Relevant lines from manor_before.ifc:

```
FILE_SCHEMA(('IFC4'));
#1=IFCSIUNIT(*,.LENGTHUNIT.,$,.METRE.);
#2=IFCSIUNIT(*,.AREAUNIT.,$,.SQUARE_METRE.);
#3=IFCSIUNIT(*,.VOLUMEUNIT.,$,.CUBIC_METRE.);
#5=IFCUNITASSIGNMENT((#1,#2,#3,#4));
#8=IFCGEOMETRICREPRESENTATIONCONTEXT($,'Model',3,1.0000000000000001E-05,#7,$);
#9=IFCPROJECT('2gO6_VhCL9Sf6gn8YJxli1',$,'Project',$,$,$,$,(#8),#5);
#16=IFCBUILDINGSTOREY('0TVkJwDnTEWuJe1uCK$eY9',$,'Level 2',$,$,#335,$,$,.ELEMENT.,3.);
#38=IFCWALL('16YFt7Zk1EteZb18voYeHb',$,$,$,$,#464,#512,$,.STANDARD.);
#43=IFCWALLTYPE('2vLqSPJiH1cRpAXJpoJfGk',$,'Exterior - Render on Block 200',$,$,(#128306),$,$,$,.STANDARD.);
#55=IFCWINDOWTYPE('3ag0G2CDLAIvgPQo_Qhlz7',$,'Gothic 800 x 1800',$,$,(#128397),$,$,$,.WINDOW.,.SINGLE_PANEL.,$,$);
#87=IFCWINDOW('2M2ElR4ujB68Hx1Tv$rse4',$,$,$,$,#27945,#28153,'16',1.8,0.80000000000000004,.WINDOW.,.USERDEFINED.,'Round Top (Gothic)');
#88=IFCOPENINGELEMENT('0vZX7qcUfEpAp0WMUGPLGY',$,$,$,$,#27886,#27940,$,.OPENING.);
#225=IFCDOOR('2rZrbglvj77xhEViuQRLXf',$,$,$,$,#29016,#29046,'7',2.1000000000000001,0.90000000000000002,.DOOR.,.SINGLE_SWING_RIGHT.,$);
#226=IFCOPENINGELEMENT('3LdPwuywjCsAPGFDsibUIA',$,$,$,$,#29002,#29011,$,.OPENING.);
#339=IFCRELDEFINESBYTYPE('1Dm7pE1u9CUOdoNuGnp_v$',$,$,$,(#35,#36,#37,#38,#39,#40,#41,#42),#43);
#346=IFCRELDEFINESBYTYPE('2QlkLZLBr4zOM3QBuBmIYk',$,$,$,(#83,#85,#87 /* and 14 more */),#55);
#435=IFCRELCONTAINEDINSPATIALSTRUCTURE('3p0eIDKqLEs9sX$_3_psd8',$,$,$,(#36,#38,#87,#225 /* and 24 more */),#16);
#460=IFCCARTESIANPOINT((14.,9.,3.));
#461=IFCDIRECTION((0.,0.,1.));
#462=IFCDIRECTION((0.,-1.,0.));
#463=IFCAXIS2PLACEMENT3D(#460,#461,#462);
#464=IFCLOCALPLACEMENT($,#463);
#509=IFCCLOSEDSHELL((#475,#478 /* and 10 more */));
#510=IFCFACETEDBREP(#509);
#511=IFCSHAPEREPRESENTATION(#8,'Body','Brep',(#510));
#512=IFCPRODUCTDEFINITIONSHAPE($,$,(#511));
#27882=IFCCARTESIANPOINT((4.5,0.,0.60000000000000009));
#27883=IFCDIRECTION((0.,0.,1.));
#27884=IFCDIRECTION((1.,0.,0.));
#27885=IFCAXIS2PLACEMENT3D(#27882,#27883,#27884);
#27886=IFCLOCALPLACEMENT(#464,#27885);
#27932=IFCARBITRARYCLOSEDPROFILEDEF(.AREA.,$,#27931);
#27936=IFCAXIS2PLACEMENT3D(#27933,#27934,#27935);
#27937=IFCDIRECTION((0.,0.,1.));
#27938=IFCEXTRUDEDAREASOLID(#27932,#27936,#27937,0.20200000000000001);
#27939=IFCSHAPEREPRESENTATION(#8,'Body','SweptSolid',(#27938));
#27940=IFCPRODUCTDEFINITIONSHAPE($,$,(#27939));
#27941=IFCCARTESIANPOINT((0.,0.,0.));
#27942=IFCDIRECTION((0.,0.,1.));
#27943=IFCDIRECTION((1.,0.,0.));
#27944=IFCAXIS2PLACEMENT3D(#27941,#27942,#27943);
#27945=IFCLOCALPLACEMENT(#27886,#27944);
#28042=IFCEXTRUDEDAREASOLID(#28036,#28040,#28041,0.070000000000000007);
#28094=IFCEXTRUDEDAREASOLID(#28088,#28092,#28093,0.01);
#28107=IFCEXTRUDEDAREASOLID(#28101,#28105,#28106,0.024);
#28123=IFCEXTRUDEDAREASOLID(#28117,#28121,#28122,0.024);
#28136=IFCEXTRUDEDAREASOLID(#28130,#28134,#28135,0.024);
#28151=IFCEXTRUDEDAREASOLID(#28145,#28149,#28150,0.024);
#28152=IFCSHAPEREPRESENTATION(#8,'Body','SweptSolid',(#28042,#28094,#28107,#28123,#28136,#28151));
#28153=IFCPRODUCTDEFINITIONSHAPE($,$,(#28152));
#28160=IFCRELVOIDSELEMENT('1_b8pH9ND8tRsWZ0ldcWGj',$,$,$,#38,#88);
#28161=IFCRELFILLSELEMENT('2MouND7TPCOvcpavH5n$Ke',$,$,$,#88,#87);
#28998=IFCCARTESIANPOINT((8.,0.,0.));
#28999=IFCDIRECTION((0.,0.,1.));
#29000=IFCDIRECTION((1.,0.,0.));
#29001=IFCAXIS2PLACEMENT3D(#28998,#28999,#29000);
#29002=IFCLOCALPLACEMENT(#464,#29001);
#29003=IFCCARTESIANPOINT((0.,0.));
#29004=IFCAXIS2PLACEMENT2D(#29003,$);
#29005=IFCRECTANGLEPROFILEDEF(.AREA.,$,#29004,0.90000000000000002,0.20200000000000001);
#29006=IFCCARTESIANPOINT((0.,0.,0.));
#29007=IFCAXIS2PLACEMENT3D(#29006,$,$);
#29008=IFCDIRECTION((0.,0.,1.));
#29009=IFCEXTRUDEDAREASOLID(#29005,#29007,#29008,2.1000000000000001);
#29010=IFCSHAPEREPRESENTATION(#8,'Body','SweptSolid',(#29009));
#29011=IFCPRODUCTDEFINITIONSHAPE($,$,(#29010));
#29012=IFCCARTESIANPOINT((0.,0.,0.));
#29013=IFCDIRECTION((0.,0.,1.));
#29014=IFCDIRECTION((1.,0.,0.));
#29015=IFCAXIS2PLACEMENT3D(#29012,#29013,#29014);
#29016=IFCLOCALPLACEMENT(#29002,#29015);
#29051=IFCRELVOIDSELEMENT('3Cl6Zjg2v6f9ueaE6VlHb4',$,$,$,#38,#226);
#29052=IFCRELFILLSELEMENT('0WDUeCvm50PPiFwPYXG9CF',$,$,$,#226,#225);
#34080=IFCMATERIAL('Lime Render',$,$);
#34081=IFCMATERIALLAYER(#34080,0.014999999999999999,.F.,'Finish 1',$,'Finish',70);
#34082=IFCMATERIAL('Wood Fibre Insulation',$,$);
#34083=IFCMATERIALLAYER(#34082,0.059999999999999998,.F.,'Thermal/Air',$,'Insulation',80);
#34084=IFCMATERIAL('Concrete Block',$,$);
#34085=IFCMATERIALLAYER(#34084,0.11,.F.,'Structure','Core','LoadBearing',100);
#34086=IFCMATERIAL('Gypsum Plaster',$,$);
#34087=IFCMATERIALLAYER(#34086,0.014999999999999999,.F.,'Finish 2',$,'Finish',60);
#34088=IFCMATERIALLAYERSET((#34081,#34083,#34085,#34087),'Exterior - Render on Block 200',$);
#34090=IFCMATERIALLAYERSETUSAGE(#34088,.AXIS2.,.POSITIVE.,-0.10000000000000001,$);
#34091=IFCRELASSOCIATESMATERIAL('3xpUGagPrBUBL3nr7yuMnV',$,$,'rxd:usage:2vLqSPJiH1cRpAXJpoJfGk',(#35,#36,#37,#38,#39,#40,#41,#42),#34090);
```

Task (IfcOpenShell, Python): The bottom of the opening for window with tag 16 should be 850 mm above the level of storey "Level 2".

```python
import numpy as np
import ifcopenshell
import ifcopenshell.api.geometry
import ifcopenshell.geom
import ifcopenshell.util.element
import ifcopenshell.util.placement
import ifcopenshell.util.shape
import ifcopenshell.util.unit

model = ifcopenshell.open("manor_before.ifc")
unit_scale = ifcopenshell.util.unit.calculate_unit_scale(model)

window = model.by_guid("2M2ElR4ujB68Hx1Tv$rse4")
opening = window.FillsVoids[0].RelatingOpeningElement
storey = ifcopenshell.util.element.get_container(window, ifc_class="IfcBuildingStorey")
level = ifcopenshell.util.placement.get_local_placement(storey.ObjectPlacement)[2, 3]

# The opening's origin need not be at the sill, so measure its lowest point.
shape = ifcopenshell.geom.create_shape(ifcopenshell.geom.settings(), opening)
bottom = ifcopenshell.util.shape.get_shape_bottom_elevation(shape, shape.geometry) / unit_scale
dz = level + 0.85 - bottom

shift = np.array([0.0, 0.0, dz])
# The window is placed relative to its opening, so it follows when the opening moves.
matrix = ifcopenshell.util.placement.get_local_placement(opening.ObjectPlacement)
matrix[:3, 3] += shift
ifcopenshell.api.geometry.edit_object_placement(
    model, product=opening, matrix=matrix, is_si=False, should_transform_children=True
)

print(f"moved by {dz * unit_scale:+.3f} m")

model.write("manor_before_updated.ifc")
```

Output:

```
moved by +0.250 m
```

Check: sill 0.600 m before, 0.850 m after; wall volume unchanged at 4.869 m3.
